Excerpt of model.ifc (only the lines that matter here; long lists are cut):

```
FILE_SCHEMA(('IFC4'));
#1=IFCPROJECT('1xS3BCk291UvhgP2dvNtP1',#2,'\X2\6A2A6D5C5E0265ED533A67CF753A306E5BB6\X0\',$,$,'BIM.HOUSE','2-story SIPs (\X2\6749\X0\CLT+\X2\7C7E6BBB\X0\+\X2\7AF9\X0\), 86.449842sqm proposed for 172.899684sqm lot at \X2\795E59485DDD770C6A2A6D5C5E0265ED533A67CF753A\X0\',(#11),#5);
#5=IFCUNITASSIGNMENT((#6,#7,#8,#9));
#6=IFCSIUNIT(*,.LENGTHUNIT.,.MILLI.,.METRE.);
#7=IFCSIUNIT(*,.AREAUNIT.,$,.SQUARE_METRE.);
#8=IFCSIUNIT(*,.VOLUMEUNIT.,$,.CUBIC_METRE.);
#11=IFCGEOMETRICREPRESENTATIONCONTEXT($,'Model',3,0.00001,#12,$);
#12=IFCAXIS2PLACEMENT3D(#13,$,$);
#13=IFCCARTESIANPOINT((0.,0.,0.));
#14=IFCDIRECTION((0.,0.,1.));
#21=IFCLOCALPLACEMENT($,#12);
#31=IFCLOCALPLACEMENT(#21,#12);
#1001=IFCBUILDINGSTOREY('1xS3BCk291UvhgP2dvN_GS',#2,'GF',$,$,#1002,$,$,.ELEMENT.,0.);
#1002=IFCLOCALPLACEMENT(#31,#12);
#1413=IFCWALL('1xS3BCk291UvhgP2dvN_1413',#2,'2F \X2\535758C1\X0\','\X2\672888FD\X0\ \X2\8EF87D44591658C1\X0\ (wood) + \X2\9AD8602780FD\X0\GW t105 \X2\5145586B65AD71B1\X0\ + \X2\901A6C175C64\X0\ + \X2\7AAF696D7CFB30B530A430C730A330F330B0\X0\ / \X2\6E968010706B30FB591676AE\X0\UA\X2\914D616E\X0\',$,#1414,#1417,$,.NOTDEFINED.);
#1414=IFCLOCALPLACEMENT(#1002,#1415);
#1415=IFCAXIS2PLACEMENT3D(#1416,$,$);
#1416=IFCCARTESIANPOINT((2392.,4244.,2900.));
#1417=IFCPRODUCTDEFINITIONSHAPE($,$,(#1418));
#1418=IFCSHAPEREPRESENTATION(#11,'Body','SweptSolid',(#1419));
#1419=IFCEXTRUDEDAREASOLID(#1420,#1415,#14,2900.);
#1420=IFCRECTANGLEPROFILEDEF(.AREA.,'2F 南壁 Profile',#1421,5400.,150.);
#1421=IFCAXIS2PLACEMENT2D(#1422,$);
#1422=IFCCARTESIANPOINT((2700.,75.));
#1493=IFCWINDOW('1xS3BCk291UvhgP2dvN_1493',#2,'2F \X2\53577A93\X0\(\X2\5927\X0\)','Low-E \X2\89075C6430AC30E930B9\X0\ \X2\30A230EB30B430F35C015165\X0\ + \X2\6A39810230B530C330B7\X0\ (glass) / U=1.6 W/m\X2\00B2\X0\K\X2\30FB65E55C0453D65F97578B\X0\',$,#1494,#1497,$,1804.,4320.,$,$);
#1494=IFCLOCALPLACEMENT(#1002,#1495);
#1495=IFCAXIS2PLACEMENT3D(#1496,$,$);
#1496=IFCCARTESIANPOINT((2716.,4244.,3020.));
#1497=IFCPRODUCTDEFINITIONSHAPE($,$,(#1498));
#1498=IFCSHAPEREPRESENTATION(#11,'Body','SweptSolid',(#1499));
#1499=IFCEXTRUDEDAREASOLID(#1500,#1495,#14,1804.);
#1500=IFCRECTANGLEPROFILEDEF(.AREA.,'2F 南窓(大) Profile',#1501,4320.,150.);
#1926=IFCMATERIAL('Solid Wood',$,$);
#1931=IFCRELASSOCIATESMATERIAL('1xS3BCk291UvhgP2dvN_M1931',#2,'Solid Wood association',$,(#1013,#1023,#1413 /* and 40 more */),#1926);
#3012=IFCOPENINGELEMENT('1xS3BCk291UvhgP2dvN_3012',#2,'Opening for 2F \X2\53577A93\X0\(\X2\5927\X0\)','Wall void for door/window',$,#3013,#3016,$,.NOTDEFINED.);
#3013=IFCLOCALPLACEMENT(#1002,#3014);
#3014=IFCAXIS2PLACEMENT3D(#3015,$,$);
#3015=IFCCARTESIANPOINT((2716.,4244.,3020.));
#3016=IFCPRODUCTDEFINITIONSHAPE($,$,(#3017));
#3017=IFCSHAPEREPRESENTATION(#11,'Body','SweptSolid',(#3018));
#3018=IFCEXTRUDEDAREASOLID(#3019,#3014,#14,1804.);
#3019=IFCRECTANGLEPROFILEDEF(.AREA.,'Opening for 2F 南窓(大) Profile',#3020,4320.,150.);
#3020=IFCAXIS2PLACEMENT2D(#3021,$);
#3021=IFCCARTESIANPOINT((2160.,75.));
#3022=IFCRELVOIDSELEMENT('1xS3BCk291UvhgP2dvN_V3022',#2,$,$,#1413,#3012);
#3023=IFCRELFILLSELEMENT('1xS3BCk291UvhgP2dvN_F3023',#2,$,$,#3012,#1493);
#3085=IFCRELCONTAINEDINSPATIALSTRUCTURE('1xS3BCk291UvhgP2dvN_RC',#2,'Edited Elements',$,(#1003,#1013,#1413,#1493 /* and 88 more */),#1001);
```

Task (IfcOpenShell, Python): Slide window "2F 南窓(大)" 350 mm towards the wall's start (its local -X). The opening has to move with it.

```python
import ifcopenshell
import ifcopenshell.api.geometry
import ifcopenshell.util.placement
import ifcopenshell.util.unit

model = ifcopenshell.open("model.ifc")
unit_scale = ifcopenshell.util.unit.calculate_unit_scale(model)

window = model.by_guid("1xS3BCk291UvhgP2dvN_1493")
opening = window.FillsVoids[0].RelatingOpeningElement
wall = opening.VoidsElements[0].RelatingBuildingElement

wall_matrix = ifcopenshell.util.placement.get_local_placement(wall.ObjectPlacement)
shift = wall_matrix[:3, 0] * -0.35 / unit_scale
before = ifcopenshell.util.placement.get_local_placement(window.ObjectPlacement)[:3, 3].copy()

# The window is not placed relative to its opening, so move both.
for product in (opening, window):
    matrix = ifcopenshell.util.placement.get_local_placement(product.ObjectPlacement)
    matrix[:3, 3] += shift
    ifcopenshell.api.geometry.edit_object_placement(model, product=product, matrix=matrix, is_si=False)

after = ifcopenshell.util.placement.get_local_placement(window.ObjectPlacement)[:3, 3]
print("window moved by", (after - before).round(3) + 0.0)

model.write("model_v2.ifc")
```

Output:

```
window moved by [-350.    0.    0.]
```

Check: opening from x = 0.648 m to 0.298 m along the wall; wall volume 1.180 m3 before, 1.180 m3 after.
